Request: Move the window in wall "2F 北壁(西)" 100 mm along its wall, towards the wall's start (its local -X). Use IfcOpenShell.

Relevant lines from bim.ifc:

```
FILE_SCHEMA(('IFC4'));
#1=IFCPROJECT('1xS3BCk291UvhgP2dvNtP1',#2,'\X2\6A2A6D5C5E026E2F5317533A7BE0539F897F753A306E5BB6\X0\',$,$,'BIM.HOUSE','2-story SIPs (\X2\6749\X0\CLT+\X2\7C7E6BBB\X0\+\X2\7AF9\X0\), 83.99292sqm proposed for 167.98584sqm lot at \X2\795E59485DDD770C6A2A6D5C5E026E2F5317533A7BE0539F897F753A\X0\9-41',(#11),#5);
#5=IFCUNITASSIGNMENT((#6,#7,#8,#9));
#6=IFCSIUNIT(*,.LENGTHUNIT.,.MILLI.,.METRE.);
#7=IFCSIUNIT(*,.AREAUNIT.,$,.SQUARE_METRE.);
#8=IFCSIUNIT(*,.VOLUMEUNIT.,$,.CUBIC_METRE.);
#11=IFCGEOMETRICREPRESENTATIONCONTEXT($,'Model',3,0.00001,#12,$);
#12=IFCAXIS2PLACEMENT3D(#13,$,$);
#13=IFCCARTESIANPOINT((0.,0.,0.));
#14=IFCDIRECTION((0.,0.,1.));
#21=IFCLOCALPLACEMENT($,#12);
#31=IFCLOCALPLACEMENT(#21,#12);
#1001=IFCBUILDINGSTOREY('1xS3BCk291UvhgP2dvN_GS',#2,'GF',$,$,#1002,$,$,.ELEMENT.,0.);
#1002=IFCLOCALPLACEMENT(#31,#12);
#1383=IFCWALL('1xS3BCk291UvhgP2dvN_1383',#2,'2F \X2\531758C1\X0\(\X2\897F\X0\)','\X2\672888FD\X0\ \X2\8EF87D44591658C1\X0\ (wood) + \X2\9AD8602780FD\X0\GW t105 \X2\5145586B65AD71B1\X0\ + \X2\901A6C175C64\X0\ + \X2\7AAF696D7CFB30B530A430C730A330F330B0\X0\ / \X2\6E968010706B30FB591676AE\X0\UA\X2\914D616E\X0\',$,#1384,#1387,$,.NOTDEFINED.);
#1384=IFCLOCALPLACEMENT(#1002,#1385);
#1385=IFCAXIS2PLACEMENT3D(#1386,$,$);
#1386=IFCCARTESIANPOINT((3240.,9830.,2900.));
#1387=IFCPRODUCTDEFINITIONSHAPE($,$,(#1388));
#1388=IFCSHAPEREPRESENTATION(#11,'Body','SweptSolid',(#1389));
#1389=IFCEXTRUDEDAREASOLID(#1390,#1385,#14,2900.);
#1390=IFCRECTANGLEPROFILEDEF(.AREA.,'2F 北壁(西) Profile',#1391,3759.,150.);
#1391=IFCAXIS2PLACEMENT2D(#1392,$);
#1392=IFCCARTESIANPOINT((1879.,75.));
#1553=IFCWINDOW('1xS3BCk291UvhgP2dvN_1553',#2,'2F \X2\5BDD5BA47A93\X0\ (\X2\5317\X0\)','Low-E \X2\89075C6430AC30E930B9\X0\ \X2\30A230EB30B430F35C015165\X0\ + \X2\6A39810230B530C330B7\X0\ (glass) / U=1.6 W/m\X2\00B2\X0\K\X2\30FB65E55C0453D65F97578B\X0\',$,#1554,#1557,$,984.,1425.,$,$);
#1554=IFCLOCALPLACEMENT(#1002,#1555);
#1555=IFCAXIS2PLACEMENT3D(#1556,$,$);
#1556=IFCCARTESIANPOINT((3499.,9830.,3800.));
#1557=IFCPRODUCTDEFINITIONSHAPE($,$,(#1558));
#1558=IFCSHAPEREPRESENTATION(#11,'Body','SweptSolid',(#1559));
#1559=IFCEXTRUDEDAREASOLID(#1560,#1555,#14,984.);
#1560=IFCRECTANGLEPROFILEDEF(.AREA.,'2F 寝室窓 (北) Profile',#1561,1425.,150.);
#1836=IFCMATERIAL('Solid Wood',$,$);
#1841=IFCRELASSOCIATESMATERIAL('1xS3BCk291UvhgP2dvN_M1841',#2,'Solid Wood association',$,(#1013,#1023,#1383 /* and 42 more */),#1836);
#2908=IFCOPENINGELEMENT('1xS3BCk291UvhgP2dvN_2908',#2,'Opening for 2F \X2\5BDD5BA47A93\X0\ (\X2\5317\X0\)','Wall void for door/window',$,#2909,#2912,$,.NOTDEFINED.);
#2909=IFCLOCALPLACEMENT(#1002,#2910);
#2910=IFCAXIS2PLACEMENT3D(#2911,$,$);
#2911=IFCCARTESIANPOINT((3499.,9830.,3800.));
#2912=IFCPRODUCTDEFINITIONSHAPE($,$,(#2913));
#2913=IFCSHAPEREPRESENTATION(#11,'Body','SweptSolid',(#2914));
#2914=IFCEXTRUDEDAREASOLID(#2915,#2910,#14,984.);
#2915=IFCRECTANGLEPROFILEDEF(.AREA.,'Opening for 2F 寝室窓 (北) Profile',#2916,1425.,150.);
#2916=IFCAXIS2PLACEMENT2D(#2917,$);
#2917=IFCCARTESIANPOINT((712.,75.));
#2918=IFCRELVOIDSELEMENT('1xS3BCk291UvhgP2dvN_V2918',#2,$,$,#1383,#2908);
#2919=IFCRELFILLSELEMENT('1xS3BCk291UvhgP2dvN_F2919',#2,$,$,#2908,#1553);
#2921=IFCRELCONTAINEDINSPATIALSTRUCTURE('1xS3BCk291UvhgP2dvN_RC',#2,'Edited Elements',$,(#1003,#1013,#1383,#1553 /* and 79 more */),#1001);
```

```python
import ifcopenshell
import ifcopenshell.api.geometry
import ifcopenshell.util.placement

model = ifcopenshell.open("bim.ifc")

window = model.by_guid("1xS3BCk291UvhgP2dvN_1553")
opening = window.FillsVoids[0].RelatingOpeningElement
wall = opening.VoidsElements[0].RelatingBuildingElement

wall_matrix = ifcopenshell.util.placement.get_local_placement(wall.ObjectPlacement)
shift = wall_matrix[:3, 0] * -100.0
before = ifcopenshell.util.placement.get_local_placement(window.ObjectPlacement)[:3, 3].copy()

# The window is not placed relative to its opening, so move both.
for product in (opening, window):
    matrix = ifcopenshell.util.placement.get_local_placement(product.ObjectPlacement)
    matrix[:3, 3] += shift
    ifcopenshell.api.geometry.edit_object_placement(model, product=product, matrix=matrix, is_si=False)

after = ifcopenshell.util.placement.get_local_placement(window.ObjectPlacement)[:3, 3]
print("window moved by", (after - before).round(3) + 0.0)

model.write("bim_updated.ifc")
```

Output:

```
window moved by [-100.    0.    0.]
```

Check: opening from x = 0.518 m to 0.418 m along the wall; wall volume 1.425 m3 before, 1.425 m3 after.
